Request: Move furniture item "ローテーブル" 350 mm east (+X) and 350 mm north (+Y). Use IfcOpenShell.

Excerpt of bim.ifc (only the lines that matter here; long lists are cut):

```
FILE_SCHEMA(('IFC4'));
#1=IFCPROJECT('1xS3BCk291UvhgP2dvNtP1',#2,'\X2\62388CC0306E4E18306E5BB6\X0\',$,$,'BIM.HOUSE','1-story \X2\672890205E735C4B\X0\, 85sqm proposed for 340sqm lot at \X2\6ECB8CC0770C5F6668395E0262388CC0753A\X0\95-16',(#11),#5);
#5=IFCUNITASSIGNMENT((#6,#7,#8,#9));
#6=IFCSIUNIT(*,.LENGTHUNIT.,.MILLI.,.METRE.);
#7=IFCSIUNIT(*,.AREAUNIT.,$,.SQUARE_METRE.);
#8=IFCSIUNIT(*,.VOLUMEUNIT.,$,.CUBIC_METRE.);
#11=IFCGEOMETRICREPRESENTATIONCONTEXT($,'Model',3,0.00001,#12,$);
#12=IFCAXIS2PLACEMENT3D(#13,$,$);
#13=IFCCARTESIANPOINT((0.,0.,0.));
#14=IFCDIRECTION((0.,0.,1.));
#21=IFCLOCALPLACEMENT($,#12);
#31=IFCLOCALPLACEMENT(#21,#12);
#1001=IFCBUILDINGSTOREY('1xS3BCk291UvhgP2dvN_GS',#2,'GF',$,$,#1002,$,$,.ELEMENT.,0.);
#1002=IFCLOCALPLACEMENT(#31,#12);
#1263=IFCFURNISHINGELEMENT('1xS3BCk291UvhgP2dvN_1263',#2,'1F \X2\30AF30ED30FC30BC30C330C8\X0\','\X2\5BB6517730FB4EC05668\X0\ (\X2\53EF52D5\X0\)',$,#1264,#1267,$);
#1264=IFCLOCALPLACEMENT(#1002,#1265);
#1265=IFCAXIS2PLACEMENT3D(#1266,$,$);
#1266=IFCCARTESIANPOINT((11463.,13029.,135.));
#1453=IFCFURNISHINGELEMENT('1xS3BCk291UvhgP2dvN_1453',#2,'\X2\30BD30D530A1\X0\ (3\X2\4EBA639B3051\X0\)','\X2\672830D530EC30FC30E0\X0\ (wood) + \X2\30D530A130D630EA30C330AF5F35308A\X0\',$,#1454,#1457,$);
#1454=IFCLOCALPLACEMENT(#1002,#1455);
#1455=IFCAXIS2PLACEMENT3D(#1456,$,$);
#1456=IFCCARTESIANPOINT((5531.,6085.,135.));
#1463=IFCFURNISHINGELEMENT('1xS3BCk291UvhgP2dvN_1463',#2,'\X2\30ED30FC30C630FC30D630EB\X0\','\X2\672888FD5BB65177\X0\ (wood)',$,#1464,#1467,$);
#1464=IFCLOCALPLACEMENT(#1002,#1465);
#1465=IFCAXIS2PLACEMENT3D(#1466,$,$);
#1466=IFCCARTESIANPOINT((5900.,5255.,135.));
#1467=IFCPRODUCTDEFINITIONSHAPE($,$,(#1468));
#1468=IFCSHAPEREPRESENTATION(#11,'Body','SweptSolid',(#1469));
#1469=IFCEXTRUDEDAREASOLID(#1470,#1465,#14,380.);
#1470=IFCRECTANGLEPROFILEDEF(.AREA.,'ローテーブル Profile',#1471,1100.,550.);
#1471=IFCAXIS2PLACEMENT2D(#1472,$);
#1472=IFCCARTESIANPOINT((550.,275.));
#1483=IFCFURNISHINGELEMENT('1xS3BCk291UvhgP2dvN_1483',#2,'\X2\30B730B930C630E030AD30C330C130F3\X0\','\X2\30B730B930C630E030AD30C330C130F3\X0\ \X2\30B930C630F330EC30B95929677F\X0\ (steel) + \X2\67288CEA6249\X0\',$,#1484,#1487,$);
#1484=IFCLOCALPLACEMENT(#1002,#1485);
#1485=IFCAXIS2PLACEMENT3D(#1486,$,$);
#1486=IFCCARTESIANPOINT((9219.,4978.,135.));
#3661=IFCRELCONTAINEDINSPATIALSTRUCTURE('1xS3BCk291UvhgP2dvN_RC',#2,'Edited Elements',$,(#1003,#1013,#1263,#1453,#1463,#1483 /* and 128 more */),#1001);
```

```python
import ifcopenshell
import ifcopenshell.api.geometry
import ifcopenshell.util.placement
import ifcopenshell.util.unit

model = ifcopenshell.open("bim.ifc")
unit_scale = ifcopenshell.util.unit.calculate_unit_scale(model)

item = model.by_guid("1xS3BCk291UvhgP2dvN_1463")
matrix = ifcopenshell.util.placement.get_local_placement(item.ObjectPlacement)
matrix[0, 3] += 0.35 / unit_scale
matrix[1, 3] += 0.35 / unit_scale
ifcopenshell.api.geometry.edit_object_placement(model, product=item, matrix=matrix, is_si=False)

print(ifcopenshell.util.placement.get_local_placement(item.ObjectPlacement).round(3) + 0.0)

model.write("bim_v2.ifc")
```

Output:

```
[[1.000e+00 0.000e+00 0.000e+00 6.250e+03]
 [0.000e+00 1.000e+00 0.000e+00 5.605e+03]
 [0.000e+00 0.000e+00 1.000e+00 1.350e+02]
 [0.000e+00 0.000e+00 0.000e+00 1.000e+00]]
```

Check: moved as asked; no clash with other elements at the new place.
